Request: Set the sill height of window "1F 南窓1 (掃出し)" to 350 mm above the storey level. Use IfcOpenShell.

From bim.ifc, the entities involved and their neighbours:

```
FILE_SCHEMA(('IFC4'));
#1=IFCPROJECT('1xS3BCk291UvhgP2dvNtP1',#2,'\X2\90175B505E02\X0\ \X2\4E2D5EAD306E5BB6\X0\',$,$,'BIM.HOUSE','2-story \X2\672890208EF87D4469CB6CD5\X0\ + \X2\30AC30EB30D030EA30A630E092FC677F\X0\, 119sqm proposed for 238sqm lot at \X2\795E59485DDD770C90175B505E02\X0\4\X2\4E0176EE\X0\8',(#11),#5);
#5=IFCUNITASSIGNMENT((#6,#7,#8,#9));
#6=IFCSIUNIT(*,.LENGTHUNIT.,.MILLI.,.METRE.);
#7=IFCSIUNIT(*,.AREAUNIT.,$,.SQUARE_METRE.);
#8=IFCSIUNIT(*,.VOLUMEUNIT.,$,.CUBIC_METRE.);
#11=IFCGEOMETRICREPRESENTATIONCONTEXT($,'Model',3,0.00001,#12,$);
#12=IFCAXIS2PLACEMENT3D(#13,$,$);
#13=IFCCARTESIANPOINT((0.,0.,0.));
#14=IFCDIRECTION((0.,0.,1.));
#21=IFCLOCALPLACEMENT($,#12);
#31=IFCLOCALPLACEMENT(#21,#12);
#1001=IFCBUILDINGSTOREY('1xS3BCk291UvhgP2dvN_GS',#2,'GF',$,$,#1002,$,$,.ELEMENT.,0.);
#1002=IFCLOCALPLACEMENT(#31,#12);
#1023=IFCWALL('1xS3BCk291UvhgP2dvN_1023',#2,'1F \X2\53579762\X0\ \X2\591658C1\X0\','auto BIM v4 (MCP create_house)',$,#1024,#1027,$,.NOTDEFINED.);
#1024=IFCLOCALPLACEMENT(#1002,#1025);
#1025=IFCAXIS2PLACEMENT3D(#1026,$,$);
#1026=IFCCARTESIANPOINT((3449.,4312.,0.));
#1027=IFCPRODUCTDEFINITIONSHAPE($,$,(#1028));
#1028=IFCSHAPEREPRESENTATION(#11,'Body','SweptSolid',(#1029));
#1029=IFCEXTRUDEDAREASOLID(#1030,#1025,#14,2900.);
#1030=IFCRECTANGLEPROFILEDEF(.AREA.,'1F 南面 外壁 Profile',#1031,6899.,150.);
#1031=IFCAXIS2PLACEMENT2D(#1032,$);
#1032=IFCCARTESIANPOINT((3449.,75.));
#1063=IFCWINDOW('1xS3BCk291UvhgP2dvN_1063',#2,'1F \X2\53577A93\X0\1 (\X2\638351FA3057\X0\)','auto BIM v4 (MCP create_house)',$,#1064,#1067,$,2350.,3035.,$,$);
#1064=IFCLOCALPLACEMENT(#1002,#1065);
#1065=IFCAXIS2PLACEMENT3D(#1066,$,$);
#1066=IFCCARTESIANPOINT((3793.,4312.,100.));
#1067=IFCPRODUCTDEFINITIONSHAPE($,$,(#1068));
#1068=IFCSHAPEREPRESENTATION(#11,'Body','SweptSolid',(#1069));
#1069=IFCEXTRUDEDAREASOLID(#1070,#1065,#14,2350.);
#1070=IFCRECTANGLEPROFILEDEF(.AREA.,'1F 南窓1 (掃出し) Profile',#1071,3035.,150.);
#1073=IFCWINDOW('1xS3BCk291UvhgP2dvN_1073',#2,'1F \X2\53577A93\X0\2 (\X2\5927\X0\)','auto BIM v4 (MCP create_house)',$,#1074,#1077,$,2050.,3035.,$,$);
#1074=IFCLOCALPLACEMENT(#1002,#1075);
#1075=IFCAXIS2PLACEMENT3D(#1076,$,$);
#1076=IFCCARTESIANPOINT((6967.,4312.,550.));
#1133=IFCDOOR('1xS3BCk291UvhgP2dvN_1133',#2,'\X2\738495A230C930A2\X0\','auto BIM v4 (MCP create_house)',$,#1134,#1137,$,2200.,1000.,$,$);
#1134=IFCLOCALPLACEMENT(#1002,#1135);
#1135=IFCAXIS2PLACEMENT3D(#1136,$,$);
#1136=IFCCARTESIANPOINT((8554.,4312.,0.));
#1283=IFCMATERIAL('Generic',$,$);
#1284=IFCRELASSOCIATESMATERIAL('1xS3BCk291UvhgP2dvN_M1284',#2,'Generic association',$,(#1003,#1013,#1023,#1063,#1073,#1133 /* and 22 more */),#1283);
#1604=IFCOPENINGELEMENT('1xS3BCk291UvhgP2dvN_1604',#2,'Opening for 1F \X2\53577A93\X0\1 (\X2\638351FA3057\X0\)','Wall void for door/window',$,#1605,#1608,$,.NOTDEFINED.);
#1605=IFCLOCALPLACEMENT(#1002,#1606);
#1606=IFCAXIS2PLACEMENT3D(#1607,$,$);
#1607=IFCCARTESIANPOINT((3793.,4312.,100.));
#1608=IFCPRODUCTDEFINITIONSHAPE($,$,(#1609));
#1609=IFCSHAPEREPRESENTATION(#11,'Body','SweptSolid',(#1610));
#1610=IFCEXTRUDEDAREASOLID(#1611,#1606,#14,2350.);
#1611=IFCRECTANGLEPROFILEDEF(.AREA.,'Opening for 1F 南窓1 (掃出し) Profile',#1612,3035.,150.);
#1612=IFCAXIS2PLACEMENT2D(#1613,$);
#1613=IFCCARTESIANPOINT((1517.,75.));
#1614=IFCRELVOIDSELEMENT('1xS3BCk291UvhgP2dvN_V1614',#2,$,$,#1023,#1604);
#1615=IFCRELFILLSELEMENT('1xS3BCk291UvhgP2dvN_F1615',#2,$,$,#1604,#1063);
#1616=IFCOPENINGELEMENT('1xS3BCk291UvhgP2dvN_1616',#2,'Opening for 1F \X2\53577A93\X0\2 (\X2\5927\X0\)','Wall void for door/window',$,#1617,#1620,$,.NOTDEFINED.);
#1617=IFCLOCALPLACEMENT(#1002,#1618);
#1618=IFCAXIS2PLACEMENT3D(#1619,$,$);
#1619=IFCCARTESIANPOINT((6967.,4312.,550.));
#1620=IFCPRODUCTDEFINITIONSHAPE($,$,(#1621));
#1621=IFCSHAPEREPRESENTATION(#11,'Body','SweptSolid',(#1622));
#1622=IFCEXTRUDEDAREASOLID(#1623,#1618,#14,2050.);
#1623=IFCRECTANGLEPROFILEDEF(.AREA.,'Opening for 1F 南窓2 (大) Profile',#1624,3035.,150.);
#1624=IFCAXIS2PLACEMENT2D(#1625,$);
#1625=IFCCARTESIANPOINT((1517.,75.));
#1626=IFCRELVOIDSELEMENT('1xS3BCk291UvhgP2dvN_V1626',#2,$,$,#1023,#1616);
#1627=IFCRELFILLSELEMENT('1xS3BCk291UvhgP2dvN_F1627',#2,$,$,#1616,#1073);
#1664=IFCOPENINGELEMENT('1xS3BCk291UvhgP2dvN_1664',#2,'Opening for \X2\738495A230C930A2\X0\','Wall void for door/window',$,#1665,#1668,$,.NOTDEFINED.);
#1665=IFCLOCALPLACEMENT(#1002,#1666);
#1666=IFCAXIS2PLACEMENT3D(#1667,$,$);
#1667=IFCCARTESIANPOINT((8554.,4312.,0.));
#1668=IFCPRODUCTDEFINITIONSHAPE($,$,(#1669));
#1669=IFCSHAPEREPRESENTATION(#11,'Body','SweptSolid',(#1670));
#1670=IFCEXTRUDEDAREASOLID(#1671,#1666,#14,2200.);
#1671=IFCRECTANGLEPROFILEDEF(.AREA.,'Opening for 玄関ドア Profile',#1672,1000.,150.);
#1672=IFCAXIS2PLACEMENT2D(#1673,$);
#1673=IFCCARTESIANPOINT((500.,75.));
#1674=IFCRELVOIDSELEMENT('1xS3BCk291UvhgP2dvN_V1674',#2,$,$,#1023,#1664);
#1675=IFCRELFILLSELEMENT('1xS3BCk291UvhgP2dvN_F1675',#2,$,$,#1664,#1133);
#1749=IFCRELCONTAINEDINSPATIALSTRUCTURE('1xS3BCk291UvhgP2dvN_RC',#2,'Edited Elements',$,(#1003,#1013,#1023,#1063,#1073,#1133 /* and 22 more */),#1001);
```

```python
import numpy as np
import ifcopenshell
import ifcopenshell.api.geometry
import ifcopenshell.geom
import ifcopenshell.util.element
import ifcopenshell.util.placement
import ifcopenshell.util.shape
import ifcopenshell.util.unit

model = ifcopenshell.open("bim.ifc")
unit_scale = ifcopenshell.util.unit.calculate_unit_scale(model)

window = model.by_guid("1xS3BCk291UvhgP2dvN_1063")
opening = window.FillsVoids[0].RelatingOpeningElement
storey = ifcopenshell.util.element.get_container(window, ifc_class="IfcBuildingStorey")
level = ifcopenshell.util.placement.get_local_placement(storey.ObjectPlacement)[2, 3]

# The opening's origin need not be at the sill, so measure its lowest point.
shape = ifcopenshell.geom.create_shape(ifcopenshell.geom.settings(), opening)
bottom = ifcopenshell.util.shape.get_shape_bottom_elevation(shape, shape.geometry) / unit_scale
dz = level + 0.35 / unit_scale - bottom

shift = np.array([0.0, 0.0, dz])
# The window is not placed relative to its opening, so move both.
for product in (opening, window):
    matrix = ifcopenshell.util.placement.get_local_placement(product.ObjectPlacement)
    matrix[:3, 3] += shift
    ifcopenshell.api.geometry.edit_object_placement(model, product=product, matrix=matrix, is_si=False)

print(f"moved by {dz * unit_scale:+.3f} m")

model.write("bim-out.ifc")
```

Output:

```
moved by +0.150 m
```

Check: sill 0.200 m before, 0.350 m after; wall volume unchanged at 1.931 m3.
